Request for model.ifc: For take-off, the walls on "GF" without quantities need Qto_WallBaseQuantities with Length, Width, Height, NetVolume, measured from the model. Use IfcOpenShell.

First a look at what the model holds.

```python
import ifcopenshell
import ifcopenshell.util.element
import ifcopenshell.util.unit

model = ifcopenshell.open("model.ifc")
print(model.schema)
for unit_type in ("LENGTHUNIT", "AREAUNIT", "VOLUMEUNIT"):
    print(unit_type, ifcopenshell.util.unit.calculate_unit_scale(model, unit_type))
storey = next(s for s in model.by_type("IfcBuildingStorey") if s.Name == "GF")
walls = [e for e in ifcopenshell.util.element.get_decomposition(storey) if e.is_a("IfcWall")]
for e in sorted(walls, key=lambda e: e.id()):
    print(e.id(), e.is_a(), e.Name, list(ifcopenshell.util.element.get_psets(e, qtos_only=True)), sep=" | ")
```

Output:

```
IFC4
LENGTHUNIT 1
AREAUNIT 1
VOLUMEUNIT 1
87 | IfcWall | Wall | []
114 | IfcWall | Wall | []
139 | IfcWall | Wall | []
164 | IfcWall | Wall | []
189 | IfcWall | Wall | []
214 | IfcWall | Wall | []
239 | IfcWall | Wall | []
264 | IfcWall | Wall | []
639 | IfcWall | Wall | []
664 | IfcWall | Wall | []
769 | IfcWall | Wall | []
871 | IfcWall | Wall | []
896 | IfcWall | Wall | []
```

```python
import ifcopenshell
import ifcopenshell.api.pset
import ifcopenshell.geom
import ifcopenshell.util.element
import ifcopenshell.util.shape
import ifcopenshell.util.unit

model = ifcopenshell.open("model.ifc")
unit_scale = ifcopenshell.util.unit.calculate_unit_scale(model)
volume_scale = ifcopenshell.util.unit.calculate_unit_scale(model, "VOLUMEUNIT")
settings = ifcopenshell.geom.settings()

storey = next(s for s in model.by_type("IfcBuildingStorey") if s.Name == "GF")
walls = [e for e in ifcopenshell.util.element.get_decomposition(storey) if e.is_a("IfcWall")]

for e in sorted(walls, key=lambda e: e.id()):
    if ifcopenshell.util.element.get_psets(e, qtos_only=True, should_inherit=False):
        continue
    # Geometry comes back in metres, in the element's own axes.
    shape = ifcopenshell.geom.create_shape(settings, e)
    values = {
        "Length": ifcopenshell.util.shape.get_x(shape.geometry) / unit_scale,
        "Width": ifcopenshell.util.shape.get_y(shape.geometry) / unit_scale,
        "Height": ifcopenshell.util.shape.get_z(shape.geometry) / unit_scale,
        "NetVolume": ifcopenshell.util.shape.get_volume(shape.geometry) / volume_scale,
    }
    qto = ifcopenshell.api.pset.add_qto(model, product=e, name="Qto_WallBaseQuantities")
    ifcopenshell.api.pset.edit_qto(model, qto=qto, properties=values)
    print(e.id(), {k: round(v, 3) for k, v in values.items()})

model.write("model_rev.ifc")
```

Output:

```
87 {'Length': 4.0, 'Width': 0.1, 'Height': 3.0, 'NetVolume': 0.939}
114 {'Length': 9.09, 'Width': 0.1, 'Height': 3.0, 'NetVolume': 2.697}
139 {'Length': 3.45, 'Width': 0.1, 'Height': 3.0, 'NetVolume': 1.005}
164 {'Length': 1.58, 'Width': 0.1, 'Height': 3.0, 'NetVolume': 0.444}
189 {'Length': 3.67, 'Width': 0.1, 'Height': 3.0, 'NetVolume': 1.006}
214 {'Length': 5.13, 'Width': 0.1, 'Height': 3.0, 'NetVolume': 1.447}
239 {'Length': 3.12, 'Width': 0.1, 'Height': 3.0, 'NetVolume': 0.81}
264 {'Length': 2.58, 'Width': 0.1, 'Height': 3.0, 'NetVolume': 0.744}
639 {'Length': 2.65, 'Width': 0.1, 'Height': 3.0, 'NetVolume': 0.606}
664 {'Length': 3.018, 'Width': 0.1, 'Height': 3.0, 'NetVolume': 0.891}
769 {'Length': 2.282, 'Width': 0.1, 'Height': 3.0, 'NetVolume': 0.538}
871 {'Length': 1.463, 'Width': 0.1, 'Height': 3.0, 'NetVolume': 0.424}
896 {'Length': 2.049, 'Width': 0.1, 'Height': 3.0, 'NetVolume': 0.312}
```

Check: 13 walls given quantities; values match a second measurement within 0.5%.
